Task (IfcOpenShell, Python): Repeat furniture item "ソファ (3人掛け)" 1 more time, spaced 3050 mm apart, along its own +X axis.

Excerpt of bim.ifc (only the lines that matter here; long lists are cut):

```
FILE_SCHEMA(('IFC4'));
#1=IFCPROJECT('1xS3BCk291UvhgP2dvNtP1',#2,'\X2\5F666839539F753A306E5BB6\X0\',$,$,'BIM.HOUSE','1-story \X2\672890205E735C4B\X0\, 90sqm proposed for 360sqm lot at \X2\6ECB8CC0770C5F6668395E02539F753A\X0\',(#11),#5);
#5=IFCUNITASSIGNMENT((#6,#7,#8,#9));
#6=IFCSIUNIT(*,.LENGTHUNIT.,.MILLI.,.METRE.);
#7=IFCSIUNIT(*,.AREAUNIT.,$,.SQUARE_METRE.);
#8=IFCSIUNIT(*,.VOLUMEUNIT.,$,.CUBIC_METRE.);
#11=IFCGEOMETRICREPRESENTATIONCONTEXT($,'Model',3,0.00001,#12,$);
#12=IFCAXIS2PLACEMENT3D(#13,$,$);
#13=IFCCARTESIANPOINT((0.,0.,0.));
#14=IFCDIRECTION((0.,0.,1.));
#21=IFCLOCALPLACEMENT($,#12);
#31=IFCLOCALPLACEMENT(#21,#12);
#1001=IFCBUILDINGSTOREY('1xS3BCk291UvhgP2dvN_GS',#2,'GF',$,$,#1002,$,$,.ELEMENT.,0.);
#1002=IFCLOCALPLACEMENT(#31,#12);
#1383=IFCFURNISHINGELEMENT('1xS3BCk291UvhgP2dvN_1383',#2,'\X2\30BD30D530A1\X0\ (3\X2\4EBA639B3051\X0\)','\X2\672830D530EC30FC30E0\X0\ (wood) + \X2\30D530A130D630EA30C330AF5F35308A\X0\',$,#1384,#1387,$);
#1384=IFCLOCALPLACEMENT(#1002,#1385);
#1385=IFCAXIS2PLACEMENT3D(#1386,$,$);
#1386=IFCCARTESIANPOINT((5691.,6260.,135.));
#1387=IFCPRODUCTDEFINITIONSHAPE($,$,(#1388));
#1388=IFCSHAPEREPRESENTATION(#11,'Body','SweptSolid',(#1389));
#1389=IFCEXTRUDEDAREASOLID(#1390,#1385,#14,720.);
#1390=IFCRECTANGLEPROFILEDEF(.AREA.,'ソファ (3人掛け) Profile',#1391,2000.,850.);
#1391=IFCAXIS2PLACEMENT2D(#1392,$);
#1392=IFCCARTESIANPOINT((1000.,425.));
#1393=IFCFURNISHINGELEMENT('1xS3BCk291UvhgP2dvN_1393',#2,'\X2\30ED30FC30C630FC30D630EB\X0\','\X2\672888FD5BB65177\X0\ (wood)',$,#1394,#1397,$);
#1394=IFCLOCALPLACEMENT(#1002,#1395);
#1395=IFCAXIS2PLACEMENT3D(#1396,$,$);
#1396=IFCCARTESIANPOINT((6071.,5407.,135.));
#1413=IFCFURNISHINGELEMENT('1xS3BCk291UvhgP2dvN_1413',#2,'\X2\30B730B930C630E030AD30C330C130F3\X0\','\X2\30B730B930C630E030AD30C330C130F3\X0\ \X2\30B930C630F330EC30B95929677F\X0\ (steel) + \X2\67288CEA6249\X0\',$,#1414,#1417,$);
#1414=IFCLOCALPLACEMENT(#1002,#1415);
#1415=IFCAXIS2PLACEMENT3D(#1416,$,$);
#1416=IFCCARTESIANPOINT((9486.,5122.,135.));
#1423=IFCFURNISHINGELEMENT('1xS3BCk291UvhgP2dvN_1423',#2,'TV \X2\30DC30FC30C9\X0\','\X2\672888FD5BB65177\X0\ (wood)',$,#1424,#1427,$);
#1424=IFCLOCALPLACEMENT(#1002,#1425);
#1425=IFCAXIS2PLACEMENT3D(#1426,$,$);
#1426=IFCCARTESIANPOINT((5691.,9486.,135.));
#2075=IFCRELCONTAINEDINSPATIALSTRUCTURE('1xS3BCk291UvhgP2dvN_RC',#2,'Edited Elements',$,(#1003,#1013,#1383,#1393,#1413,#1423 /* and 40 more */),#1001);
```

```python
import ifcopenshell
import ifcopenshell.api.geometry
import ifcopenshell.api.root
import ifcopenshell.util.element
import ifcopenshell.util.placement

model = ifcopenshell.open("bim.ifc")


def reuse_history(source, copy):
    """copy_class also copies each property set's owner history, people and application; keep the originals."""
    for rel in copy.IsDefinedBy:
        if rel.is_a("IfcRelDefinesByProperties") and (history := rel.RelatingPropertyDefinition.OwnerHistory):
            rel.RelatingPropertyDefinition.OwnerHistory = source.OwnerHistory
            ifcopenshell.util.element.remove_deep2(model, history)


source = model.by_id(1383)
base = ifcopenshell.util.placement.get_local_placement(source.ObjectPlacement)
step = base[:3, 0] * 3050.0

for i in range(1, 2):
    copy = ifcopenshell.api.root.copy_class(model, product=source)
    copy.Representation = ifcopenshell.util.element.copy_deep(
        model, source.Representation, exclude=["IfcGeometricRepresentationContext", "IfcRepresentationMap"]
    )
    reuse_history(source, copy)
    matrix = base.copy()
    matrix[:3, 3] += i * step
    print("added at", matrix[:3, 3].round(3) + 0.0)
    ifcopenshell.api.geometry.edit_object_placement(model, product=copy, matrix=matrix, is_si=False)

model.write("bim_v2.ifc")
```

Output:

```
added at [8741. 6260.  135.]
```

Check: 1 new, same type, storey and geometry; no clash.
